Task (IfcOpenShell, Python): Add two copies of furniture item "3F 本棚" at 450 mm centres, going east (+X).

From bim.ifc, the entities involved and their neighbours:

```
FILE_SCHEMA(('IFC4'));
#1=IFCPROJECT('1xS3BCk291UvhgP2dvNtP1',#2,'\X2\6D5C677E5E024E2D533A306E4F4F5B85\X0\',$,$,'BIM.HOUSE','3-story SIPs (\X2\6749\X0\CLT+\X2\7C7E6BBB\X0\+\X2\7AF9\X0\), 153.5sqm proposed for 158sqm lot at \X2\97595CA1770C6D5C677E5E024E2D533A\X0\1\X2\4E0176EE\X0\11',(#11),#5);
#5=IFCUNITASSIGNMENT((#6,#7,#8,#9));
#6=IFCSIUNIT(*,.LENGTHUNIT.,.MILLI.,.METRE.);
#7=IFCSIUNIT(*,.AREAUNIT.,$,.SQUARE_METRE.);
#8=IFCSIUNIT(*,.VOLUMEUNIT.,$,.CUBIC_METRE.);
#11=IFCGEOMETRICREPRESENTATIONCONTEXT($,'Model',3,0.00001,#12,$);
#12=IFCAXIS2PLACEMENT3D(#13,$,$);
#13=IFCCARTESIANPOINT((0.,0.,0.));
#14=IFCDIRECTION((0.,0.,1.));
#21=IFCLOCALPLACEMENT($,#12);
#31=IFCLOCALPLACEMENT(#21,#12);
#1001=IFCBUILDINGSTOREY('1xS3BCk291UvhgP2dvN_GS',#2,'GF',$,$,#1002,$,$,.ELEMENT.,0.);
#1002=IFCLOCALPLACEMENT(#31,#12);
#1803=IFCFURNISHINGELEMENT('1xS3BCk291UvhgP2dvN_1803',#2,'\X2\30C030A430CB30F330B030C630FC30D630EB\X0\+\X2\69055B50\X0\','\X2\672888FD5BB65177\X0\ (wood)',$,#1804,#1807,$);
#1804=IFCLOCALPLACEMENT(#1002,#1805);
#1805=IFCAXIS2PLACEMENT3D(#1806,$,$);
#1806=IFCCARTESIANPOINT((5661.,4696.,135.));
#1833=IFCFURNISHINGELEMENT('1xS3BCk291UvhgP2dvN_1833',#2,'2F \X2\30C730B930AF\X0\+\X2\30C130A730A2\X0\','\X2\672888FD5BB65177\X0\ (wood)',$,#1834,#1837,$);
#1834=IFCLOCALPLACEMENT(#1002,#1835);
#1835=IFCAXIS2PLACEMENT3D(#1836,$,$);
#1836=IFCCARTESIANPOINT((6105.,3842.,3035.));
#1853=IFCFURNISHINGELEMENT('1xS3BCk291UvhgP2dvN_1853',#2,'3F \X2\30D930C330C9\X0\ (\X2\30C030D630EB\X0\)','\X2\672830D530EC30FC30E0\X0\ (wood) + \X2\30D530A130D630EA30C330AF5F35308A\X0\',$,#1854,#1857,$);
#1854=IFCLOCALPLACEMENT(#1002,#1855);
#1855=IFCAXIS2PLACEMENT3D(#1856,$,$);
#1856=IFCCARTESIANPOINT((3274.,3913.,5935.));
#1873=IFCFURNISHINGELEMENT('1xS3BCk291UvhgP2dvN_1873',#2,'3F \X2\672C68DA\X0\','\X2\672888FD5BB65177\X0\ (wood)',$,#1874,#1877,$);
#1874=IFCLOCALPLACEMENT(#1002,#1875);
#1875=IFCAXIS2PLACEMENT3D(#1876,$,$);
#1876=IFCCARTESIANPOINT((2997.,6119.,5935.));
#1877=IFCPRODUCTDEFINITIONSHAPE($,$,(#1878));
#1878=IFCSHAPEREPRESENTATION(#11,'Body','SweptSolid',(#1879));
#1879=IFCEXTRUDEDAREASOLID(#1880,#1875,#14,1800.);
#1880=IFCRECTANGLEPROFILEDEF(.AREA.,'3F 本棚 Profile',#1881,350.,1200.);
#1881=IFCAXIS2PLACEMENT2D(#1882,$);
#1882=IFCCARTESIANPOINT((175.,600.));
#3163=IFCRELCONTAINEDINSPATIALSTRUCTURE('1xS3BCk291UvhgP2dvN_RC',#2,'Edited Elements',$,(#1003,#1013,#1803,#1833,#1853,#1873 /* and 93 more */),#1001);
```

```python
import numpy as np
import ifcopenshell
import ifcopenshell.api.geometry
import ifcopenshell.api.root
import ifcopenshell.util.element
import ifcopenshell.util.placement

model = ifcopenshell.open("bim.ifc")


def reuse_history(source, copy):
    """copy_class also copies each property set's owner history, people and application; keep the originals."""
    for rel in copy.IsDefinedBy:
        if rel.is_a("IfcRelDefinesByProperties") and (history := rel.RelatingPropertyDefinition.OwnerHistory):
            rel.RelatingPropertyDefinition.OwnerHistory = source.OwnerHistory
            ifcopenshell.util.element.remove_deep2(model, history)


source = model.by_guid("1xS3BCk291UvhgP2dvN_1873")
base = ifcopenshell.util.placement.get_local_placement(source.ObjectPlacement)
step = np.array([1.0, 0.0, 0.0]) * 450.0

for i in range(1, 3):
    copy = ifcopenshell.api.root.copy_class(model, product=source)
    copy.Representation = ifcopenshell.util.element.copy_deep(
        model, source.Representation, exclude=["IfcGeometricRepresentationContext", "IfcRepresentationMap"]
    )
    reuse_history(source, copy)
    matrix = base.copy()
    matrix[:3, 3] += i * step
    print("added at", matrix[:3, 3].round(3) + 0.0)
    ifcopenshell.api.geometry.edit_object_placement(model, product=copy, matrix=matrix, is_si=False)

model.write("bim_v2.ifc")
```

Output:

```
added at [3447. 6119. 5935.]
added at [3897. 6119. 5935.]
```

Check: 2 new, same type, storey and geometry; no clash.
